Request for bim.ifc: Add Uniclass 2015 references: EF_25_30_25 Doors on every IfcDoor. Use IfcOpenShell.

First a look at what the model holds.

```python
import ifcopenshell

model = ifcopenshell.open("bim.ifc")
print(model.schema)
print("classifications:", [c.Name for c in model.by_type("IfcClassification")])
for ifc_class in ("IfcDoor", "IfcRoof", "IfcStair", "IfcWall", "IfcWindow"):
    print(ifc_class, len(model.by_type(ifc_class)))
```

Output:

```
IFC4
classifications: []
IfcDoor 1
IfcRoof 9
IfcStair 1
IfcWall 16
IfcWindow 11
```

```python
import ifcopenshell
import ifcopenshell.api.classification

model = ifcopenshell.open("bim.ifc")

system = ifcopenshell.api.classification.add_classification(model, classification="Uniclass 2015")

codes = {
    "IfcDoor": ("EF_25_30_25", "Doors"),
}
for ifc_class, (code, name) in codes.items():
    products = model.by_type(ifc_class)
    ifcopenshell.api.classification.add_reference(
        model, products=products, classification=system, identification=code, name=name
    )
    print(code, len(products))

model.write("bim_v2.ifc")
```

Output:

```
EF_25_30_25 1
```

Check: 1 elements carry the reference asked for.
